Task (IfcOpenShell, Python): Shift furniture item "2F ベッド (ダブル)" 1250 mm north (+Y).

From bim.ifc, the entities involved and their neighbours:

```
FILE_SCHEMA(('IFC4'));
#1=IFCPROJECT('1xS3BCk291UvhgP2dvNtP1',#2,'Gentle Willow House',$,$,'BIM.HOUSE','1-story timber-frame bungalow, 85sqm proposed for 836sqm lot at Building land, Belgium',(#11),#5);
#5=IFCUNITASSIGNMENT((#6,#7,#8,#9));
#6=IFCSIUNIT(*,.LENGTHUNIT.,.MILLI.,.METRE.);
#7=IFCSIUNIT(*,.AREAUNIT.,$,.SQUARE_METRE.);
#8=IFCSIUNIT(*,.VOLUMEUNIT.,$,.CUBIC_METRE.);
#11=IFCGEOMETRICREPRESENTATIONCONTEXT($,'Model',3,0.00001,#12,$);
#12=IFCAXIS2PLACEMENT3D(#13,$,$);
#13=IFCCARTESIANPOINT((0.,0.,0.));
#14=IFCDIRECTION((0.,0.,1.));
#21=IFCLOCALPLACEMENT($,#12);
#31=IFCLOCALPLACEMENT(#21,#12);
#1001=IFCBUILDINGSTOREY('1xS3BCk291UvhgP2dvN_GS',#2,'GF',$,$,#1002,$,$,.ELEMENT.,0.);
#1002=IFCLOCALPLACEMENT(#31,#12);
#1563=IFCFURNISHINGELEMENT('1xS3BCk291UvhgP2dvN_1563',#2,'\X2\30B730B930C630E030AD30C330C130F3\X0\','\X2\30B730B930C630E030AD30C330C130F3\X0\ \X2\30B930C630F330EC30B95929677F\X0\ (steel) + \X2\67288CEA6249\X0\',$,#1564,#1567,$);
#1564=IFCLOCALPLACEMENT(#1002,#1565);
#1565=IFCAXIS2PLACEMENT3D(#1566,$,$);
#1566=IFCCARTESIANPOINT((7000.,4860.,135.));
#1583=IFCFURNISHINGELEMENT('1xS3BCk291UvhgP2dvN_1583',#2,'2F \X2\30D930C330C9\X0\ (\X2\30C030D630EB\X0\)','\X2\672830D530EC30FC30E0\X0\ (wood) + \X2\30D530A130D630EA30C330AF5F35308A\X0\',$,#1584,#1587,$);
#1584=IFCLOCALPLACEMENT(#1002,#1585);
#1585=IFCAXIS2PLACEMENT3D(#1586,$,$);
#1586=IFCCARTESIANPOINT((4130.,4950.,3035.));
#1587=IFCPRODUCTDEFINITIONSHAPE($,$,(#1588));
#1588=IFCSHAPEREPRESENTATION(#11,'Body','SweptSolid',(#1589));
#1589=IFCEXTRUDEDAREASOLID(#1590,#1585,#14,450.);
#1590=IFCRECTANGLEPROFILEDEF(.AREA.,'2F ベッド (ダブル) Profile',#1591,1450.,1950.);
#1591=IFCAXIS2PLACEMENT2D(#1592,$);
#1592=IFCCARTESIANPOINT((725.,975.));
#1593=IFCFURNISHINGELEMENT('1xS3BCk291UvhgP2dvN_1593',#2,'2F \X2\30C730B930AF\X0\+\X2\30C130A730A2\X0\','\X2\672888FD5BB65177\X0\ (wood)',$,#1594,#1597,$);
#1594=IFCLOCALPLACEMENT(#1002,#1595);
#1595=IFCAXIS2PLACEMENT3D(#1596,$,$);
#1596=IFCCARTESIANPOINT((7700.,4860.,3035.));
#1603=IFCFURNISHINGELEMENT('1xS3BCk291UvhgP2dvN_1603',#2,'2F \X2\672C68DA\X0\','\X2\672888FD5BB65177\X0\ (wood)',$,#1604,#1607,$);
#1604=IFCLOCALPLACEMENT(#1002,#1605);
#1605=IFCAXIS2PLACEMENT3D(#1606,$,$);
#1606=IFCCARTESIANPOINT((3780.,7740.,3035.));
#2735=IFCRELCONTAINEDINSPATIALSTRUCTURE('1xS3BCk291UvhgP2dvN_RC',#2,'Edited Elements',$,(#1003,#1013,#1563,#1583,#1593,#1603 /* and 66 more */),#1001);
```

```python
import ifcopenshell
import ifcopenshell.api.geometry
import ifcopenshell.util.placement
import ifcopenshell.util.unit

model = ifcopenshell.open("bim.ifc")
unit_scale = ifcopenshell.util.unit.calculate_unit_scale(model)

item = model.by_guid("1xS3BCk291UvhgP2dvN_1583")
matrix = ifcopenshell.util.placement.get_local_placement(item.ObjectPlacement)
matrix[1, 3] += 1.25 / unit_scale
ifcopenshell.api.geometry.edit_object_placement(model, product=item, matrix=matrix, is_si=False)

print(ifcopenshell.util.placement.get_local_placement(item.ObjectPlacement).round(3) + 0.0)

model.write("bim_rev.ifc")
```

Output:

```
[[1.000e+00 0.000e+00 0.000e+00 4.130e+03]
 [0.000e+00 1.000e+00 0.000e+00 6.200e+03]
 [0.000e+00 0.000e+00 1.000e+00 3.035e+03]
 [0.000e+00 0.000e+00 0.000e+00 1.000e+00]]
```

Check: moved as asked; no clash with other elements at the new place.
